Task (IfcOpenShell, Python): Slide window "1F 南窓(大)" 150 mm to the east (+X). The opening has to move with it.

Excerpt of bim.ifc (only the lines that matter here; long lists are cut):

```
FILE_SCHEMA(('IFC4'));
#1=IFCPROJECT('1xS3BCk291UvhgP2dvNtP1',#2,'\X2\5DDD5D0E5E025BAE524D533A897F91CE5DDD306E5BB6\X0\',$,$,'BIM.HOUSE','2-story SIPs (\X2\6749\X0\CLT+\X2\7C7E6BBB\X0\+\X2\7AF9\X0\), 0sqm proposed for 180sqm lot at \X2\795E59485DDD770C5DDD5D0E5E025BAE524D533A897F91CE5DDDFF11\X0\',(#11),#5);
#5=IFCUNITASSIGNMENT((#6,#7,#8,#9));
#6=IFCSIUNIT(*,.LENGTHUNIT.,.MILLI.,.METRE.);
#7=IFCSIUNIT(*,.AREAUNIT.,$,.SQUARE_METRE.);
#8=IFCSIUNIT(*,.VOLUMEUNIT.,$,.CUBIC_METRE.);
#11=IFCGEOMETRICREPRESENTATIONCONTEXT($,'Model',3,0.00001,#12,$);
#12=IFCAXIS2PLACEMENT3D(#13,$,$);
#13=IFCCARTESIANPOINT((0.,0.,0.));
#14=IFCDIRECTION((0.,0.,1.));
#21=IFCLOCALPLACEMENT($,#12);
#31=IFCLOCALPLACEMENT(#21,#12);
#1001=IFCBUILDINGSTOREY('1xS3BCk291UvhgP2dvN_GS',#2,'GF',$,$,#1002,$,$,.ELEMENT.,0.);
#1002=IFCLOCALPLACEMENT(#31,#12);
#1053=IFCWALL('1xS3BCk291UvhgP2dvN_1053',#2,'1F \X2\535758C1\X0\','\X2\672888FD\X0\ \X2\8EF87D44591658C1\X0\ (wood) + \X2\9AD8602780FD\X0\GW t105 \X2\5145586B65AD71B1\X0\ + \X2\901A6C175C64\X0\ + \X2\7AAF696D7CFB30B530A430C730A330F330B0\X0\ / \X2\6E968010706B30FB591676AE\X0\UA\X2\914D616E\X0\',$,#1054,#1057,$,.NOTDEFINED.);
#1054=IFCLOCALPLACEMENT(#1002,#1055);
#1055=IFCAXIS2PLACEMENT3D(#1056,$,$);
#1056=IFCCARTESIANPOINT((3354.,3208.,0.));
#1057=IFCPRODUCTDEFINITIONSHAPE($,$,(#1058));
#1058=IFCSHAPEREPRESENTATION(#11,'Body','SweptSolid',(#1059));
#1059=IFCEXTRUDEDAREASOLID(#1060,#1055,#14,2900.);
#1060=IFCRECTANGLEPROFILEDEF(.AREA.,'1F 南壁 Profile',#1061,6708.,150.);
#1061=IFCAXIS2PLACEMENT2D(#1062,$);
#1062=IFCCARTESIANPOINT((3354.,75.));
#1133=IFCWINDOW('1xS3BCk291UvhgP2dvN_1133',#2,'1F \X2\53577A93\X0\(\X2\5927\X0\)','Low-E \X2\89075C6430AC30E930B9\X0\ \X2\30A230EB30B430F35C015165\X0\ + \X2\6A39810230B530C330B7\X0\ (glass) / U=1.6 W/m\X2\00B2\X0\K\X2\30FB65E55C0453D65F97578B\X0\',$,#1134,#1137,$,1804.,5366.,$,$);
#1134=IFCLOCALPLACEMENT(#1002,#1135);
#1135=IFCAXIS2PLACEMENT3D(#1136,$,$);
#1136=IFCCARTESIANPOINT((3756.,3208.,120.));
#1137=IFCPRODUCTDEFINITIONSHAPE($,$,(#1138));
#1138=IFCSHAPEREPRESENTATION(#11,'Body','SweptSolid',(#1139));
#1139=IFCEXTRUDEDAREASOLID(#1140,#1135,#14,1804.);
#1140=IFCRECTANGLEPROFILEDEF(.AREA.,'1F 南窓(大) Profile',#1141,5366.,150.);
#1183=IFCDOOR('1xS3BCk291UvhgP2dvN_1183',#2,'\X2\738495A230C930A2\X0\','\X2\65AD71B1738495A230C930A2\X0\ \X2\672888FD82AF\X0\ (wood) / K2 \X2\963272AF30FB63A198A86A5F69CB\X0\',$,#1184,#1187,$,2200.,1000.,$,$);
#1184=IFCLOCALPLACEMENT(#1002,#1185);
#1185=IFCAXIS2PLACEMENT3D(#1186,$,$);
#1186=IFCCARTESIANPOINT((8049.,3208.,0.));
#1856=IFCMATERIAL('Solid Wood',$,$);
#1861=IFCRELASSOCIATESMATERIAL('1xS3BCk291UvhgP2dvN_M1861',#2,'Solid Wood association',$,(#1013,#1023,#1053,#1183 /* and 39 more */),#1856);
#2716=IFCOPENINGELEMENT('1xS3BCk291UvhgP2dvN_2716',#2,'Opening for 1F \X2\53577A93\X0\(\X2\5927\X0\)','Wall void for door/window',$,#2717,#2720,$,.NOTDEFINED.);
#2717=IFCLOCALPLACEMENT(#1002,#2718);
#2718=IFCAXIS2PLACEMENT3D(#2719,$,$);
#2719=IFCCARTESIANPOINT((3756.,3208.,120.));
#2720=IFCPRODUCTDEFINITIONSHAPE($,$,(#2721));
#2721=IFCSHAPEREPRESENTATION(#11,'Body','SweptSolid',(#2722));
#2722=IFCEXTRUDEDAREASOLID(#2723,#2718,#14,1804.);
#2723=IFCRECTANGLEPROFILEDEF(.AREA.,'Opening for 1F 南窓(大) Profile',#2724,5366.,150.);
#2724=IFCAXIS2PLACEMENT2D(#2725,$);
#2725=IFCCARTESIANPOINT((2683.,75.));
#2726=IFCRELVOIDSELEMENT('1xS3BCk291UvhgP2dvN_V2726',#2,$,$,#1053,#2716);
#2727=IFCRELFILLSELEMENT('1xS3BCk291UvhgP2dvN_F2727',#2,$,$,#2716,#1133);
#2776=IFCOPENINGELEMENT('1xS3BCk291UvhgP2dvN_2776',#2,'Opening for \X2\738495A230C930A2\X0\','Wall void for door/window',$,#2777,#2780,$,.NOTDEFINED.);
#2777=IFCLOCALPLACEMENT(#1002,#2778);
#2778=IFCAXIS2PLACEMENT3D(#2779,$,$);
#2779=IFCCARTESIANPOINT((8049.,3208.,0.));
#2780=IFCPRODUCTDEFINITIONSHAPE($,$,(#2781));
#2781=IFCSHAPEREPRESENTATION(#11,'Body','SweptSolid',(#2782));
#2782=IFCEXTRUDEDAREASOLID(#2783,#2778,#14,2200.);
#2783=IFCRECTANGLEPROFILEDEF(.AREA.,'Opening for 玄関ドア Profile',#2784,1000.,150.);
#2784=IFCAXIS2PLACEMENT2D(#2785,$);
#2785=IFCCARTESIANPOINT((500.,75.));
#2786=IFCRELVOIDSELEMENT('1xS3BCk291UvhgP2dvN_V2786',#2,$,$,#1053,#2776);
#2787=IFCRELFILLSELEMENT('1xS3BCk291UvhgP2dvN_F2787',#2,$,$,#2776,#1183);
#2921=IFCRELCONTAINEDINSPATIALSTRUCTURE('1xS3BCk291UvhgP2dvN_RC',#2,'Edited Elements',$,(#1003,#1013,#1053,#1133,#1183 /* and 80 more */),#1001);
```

```python
import ifcopenshell
import ifcopenshell.api.geometry
import ifcopenshell.util.placement
import ifcopenshell.util.unit

model = ifcopenshell.open("bim.ifc")
unit_scale = ifcopenshell.util.unit.calculate_unit_scale(model)

window = model.by_guid("1xS3BCk291UvhgP2dvN_1133")
opening = window.FillsVoids[0].RelatingOpeningElement
wall = opening.VoidsElements[0].RelatingBuildingElement

wall_matrix = ifcopenshell.util.placement.get_local_placement(wall.ObjectPlacement)
shift = wall_matrix[:3, 0] * 0.15 / unit_scale
before = ifcopenshell.util.placement.get_local_placement(window.ObjectPlacement)[:3, 3].copy()

# The window is not placed relative to its opening, so move both.
for product in (opening, window):
    matrix = ifcopenshell.util.placement.get_local_placement(product.ObjectPlacement)
    matrix[:3, 3] += shift
    ifcopenshell.api.geometry.edit_object_placement(model, product=product, matrix=matrix, is_si=False)

after = ifcopenshell.util.placement.get_local_placement(window.ObjectPlacement)[:3, 3]
print("window moved by", (after - before).round(3) + 0.0)

model.write("bim_v2.ifc")
```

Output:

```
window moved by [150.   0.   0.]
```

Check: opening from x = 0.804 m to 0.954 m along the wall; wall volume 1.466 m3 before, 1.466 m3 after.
